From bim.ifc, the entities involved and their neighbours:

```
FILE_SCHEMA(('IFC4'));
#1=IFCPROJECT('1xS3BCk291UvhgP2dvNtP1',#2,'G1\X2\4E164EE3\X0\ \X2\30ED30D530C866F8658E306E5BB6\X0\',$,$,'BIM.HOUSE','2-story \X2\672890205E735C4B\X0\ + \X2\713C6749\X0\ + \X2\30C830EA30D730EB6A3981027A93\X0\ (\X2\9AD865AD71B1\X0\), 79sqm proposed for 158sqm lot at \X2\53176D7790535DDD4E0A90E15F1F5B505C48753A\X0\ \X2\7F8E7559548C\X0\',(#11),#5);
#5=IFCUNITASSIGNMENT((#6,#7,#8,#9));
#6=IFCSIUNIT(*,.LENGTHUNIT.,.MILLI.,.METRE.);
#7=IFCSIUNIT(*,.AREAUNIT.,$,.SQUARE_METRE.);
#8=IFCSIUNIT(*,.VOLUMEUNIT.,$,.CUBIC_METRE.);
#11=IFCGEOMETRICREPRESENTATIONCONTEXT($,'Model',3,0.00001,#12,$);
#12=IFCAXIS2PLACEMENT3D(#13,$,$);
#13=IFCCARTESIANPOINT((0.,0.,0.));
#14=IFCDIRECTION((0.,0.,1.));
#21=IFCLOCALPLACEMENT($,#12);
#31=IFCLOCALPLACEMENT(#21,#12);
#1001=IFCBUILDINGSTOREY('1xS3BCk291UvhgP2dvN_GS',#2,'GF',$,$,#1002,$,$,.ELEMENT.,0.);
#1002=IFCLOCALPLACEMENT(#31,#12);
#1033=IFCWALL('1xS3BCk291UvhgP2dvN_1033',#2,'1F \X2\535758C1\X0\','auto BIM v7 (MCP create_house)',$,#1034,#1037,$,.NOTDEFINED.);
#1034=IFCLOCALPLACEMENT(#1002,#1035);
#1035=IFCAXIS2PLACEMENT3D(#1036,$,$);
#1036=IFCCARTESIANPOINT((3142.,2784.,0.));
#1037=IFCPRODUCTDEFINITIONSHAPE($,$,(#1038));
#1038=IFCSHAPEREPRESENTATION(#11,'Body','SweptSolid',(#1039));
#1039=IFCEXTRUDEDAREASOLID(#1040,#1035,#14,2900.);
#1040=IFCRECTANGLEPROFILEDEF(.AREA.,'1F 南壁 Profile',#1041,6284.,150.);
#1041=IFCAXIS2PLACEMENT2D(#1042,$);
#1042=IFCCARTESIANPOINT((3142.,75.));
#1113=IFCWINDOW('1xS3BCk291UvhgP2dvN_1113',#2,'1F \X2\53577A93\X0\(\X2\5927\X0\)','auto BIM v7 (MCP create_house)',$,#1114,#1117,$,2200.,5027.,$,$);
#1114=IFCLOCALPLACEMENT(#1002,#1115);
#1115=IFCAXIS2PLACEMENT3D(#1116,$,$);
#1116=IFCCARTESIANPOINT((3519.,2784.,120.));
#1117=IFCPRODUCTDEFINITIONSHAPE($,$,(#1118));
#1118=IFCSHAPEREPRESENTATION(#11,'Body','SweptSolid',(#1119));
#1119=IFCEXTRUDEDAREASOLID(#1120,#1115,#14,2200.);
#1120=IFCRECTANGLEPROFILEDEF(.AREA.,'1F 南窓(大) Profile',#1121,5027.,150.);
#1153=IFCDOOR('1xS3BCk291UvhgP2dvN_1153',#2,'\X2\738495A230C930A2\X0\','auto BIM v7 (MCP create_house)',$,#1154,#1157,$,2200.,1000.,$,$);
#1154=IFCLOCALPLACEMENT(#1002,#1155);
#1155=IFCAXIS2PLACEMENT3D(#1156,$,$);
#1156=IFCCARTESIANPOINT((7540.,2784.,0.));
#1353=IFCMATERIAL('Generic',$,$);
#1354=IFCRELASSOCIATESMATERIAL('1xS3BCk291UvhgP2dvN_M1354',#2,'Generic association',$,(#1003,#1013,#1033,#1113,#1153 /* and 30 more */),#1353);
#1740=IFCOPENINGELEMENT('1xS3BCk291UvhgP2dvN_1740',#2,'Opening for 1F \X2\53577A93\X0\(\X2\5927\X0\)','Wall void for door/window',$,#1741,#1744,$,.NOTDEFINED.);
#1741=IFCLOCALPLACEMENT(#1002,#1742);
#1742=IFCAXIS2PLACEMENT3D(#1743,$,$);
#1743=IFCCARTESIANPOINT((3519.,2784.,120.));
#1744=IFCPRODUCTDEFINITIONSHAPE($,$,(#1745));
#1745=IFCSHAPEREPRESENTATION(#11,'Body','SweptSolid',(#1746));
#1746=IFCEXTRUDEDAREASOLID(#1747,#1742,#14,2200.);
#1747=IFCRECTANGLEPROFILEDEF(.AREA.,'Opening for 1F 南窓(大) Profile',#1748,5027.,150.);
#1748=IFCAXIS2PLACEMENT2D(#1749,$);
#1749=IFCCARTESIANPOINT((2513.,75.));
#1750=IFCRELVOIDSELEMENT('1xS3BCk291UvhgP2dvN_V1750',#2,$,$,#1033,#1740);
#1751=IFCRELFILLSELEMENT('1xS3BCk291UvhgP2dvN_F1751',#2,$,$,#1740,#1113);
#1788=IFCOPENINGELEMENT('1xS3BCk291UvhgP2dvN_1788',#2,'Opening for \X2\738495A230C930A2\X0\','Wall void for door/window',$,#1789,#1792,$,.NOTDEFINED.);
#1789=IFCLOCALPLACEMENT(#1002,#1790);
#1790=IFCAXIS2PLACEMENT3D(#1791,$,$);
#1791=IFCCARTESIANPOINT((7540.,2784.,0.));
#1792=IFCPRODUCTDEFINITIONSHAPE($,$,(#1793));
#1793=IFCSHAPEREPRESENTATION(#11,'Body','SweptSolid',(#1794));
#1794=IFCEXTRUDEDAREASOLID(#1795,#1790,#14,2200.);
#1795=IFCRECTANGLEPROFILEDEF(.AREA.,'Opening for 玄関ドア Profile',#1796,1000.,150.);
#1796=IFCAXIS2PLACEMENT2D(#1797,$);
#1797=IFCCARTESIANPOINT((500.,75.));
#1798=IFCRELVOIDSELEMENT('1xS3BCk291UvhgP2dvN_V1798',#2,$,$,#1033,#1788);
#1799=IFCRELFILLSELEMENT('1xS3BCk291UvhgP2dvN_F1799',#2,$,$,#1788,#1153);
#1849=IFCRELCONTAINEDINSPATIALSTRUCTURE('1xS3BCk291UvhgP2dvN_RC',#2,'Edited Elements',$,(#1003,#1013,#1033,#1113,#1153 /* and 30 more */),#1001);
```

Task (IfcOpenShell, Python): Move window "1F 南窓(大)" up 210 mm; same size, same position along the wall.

```python
import numpy as np
import ifcopenshell
import ifcopenshell.api.geometry
import ifcopenshell.util.placement
import ifcopenshell.util.unit

model = ifcopenshell.open("bim.ifc")
unit_scale = ifcopenshell.util.unit.calculate_unit_scale(model)

window = model.by_id(1113)
opening = window.FillsVoids[0].RelatingOpeningElement
dz = 0.21 / unit_scale

shift = np.array([0.0, 0.0, dz])
# The window is not placed relative to its opening, so move both.
for product in (opening, window):
    matrix = ifcopenshell.util.placement.get_local_placement(product.ObjectPlacement)
    matrix[:3, 3] += shift
    ifcopenshell.api.geometry.edit_object_placement(model, product=product, matrix=matrix, is_si=False)

print(f"moved by {dz * unit_scale:+.3f} m")

model.write("bim_v2.ifc")
```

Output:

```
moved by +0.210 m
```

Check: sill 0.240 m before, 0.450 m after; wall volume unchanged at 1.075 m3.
